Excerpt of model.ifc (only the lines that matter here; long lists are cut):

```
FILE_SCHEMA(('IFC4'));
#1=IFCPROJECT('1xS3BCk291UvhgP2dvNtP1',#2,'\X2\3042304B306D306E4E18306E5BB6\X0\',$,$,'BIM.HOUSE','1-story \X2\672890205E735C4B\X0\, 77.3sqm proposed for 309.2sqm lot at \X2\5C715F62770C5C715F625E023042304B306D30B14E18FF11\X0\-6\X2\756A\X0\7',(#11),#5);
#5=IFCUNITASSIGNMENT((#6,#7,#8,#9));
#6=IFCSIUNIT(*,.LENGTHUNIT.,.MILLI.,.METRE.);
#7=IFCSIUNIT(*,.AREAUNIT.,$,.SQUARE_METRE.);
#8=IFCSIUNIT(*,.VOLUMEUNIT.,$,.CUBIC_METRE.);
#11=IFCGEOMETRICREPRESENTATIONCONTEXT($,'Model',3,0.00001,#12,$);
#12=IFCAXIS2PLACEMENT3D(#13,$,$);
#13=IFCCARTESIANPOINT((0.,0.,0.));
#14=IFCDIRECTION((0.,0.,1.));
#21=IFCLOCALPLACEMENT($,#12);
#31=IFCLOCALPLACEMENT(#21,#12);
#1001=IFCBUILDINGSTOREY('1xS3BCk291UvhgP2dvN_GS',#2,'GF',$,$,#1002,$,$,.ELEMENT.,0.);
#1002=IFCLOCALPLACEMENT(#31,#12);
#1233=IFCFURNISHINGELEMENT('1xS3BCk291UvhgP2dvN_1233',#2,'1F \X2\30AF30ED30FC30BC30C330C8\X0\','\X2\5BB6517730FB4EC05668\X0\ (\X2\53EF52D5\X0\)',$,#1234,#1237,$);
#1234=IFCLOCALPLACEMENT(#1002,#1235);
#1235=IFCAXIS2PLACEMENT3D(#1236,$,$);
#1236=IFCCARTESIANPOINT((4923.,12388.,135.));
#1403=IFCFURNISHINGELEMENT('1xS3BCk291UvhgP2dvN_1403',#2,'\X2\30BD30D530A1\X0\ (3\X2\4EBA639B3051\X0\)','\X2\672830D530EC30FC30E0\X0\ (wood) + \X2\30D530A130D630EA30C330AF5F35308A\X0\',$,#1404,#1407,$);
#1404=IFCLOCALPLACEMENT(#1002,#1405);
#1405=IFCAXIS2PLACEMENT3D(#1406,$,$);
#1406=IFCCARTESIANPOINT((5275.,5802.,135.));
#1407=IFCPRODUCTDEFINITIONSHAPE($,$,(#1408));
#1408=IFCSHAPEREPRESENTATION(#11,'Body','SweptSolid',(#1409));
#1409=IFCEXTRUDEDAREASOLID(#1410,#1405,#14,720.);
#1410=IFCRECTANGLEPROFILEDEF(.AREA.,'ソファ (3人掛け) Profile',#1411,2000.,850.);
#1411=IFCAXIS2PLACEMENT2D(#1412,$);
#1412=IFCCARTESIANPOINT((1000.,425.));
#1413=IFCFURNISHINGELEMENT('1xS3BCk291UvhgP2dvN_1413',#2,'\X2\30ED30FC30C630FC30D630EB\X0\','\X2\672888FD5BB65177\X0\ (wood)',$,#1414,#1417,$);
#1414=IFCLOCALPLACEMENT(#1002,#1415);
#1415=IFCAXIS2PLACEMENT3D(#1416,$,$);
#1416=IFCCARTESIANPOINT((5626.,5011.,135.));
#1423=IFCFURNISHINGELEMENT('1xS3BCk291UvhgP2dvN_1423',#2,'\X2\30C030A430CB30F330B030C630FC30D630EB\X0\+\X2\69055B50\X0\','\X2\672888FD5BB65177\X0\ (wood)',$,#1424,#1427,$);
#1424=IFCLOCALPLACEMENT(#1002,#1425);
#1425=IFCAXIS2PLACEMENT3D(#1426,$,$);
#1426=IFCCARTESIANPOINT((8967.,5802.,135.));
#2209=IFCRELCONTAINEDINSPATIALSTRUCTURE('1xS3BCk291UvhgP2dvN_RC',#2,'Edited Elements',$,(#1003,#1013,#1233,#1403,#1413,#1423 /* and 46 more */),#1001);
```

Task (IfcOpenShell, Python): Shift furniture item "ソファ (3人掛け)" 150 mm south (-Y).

```python
import ifcopenshell
import ifcopenshell.api.geometry
import ifcopenshell.util.placement
import ifcopenshell.util.unit

model = ifcopenshell.open("model.ifc")
unit_scale = ifcopenshell.util.unit.calculate_unit_scale(model)

item = model.by_guid("1xS3BCk291UvhgP2dvN_1403")
matrix = ifcopenshell.util.placement.get_local_placement(item.ObjectPlacement)
matrix[1, 3] -= 0.15 / unit_scale
ifcopenshell.api.geometry.edit_object_placement(model, product=item, matrix=matrix, is_si=False)

print(ifcopenshell.util.placement.get_local_placement(item.ObjectPlacement).round(3) + 0.0)

model.write("model_v2.ifc")
```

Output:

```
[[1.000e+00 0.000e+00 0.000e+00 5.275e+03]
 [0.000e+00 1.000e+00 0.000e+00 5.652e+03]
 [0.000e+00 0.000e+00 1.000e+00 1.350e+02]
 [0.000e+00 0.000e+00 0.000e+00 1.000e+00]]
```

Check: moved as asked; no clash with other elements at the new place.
